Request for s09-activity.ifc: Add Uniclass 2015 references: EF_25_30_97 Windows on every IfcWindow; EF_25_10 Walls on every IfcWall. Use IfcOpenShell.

First a look at what the model holds.

```python
import ifcopenshell

model = ifcopenshell.open("s09-activity.ifc")
print(model.schema)
print("classifications:", [c.Name for c in model.by_type("IfcClassification")])
for ifc_class in ("IfcDoor", "IfcRoof", "IfcStair", "IfcWall", "IfcWindow"):
    print(ifc_class, len(model.by_type(ifc_class)))
```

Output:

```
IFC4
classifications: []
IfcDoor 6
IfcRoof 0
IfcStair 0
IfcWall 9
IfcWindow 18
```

```python
import ifcopenshell
import ifcopenshell.api.classification

model = ifcopenshell.open("s09-activity.ifc")

system = ifcopenshell.api.classification.add_classification(model, classification="Uniclass 2015")

codes = {
    "IfcWindow": ("EF_25_30_97", "Windows"),
    "IfcWall": ("EF_25_10", "Walls"),
}
for ifc_class, (code, name) in codes.items():
    products = model.by_type(ifc_class)
    ifcopenshell.api.classification.add_reference(
        model, products=products, classification=system, identification=code, name=name
    )
    print(code, len(products))

model.write("s09-activity-out.ifc")
```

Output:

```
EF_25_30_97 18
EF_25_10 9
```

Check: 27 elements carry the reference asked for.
